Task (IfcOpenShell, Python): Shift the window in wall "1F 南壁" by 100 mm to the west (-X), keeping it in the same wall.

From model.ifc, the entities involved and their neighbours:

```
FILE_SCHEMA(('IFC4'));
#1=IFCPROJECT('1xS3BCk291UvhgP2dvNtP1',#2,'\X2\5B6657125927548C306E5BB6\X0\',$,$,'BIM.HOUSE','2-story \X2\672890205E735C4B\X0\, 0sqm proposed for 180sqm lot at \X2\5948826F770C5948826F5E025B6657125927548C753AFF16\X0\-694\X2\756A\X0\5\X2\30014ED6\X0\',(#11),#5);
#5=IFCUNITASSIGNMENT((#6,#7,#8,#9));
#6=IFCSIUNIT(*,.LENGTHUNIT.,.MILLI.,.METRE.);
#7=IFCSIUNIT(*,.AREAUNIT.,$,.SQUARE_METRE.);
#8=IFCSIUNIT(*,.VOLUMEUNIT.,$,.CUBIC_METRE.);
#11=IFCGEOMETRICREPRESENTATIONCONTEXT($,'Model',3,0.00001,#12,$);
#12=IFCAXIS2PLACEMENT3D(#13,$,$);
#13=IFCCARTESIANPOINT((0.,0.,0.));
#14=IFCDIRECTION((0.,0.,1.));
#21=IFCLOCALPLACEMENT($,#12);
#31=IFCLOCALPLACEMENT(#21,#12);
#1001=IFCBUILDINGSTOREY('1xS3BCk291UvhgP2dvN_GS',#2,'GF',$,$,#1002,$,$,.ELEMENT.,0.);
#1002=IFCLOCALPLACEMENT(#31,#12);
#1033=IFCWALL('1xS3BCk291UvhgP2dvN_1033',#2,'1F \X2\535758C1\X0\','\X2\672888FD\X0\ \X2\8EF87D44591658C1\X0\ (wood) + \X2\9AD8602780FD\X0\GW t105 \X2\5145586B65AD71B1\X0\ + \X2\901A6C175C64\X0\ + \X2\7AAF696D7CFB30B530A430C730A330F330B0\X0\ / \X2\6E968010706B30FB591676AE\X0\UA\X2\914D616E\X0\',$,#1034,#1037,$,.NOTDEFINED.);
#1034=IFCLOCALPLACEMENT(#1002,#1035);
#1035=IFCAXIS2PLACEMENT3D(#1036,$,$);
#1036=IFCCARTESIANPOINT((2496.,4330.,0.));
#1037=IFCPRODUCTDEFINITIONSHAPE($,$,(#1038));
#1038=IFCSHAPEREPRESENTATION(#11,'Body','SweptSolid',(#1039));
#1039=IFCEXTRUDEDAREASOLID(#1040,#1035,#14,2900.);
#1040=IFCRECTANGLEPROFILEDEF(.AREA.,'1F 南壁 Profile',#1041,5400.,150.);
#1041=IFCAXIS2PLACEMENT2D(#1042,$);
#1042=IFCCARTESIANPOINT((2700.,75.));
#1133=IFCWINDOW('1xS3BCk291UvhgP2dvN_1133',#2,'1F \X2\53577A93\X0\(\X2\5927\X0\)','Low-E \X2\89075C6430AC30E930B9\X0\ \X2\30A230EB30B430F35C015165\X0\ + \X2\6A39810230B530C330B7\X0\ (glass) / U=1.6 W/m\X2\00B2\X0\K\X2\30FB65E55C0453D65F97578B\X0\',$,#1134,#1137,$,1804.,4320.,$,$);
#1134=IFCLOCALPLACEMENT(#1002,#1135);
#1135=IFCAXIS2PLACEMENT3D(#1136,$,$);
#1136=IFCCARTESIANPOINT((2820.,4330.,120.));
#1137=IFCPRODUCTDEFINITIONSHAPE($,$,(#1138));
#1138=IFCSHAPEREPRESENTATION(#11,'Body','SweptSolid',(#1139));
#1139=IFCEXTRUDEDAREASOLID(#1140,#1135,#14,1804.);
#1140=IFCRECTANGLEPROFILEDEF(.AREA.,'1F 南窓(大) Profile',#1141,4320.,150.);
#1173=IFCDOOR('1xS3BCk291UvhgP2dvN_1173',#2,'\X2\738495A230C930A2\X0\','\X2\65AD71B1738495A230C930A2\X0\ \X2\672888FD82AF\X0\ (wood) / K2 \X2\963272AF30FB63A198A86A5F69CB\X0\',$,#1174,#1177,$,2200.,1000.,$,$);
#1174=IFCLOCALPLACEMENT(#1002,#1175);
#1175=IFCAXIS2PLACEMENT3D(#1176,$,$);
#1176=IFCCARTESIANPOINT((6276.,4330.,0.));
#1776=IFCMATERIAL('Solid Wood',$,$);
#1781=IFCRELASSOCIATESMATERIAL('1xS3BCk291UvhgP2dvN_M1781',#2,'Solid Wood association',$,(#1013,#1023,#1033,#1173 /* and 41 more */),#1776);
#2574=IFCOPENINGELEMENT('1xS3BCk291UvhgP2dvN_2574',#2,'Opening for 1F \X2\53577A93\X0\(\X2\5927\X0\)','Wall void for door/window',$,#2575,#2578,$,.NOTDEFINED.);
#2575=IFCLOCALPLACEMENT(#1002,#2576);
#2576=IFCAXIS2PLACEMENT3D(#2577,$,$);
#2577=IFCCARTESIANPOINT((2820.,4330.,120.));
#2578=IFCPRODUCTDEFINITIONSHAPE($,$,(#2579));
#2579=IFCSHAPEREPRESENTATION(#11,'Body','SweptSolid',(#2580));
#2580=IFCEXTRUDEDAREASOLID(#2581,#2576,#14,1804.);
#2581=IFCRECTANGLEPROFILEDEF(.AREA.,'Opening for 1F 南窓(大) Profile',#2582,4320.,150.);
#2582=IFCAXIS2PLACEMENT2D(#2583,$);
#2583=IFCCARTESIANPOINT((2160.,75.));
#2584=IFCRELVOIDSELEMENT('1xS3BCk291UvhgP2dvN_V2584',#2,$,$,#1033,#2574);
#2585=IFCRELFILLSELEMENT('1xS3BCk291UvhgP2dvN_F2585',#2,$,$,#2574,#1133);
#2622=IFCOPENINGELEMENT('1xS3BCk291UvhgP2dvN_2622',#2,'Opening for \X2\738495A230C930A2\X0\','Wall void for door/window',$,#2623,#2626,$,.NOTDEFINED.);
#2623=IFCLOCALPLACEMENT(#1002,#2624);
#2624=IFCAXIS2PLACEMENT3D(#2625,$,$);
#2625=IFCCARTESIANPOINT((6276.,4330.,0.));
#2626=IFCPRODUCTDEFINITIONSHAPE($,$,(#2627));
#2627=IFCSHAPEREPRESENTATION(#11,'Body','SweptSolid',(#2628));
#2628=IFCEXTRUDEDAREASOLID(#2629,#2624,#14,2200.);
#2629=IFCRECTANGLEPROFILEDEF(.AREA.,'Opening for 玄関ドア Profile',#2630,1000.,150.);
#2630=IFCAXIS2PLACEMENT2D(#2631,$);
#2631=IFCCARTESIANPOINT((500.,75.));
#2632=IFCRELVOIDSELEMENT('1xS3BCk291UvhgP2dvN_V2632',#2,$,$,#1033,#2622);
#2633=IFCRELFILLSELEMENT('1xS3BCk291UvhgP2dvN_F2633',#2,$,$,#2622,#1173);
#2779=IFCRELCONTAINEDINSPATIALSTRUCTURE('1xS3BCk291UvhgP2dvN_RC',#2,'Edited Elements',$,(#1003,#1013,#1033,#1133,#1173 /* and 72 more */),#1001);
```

```python
import ifcopenshell
import ifcopenshell.api.geometry
import ifcopenshell.util.placement

model = ifcopenshell.open("model.ifc")

window = model.by_guid("1xS3BCk291UvhgP2dvN_1133")
opening = window.FillsVoids[0].RelatingOpeningElement
wall = opening.VoidsElements[0].RelatingBuildingElement

wall_matrix = ifcopenshell.util.placement.get_local_placement(wall.ObjectPlacement)
shift = wall_matrix[:3, 0] * -100.0
before = ifcopenshell.util.placement.get_local_placement(window.ObjectPlacement)[:3, 3].copy()

# The window is not placed relative to its opening, so move both.
for product in (opening, window):
    matrix = ifcopenshell.util.placement.get_local_placement(product.ObjectPlacement)
    matrix[:3, 3] += shift
    ifcopenshell.api.geometry.edit_object_placement(model, product=product, matrix=matrix, is_si=False)

after = ifcopenshell.util.placement.get_local_placement(window.ObjectPlacement)[:3, 3]
print("window moved by", (after - before).round(3) + 0.0)

model.write("model_rev.ifc")
```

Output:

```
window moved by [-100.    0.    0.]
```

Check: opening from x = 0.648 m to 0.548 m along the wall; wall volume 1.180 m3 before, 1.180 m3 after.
